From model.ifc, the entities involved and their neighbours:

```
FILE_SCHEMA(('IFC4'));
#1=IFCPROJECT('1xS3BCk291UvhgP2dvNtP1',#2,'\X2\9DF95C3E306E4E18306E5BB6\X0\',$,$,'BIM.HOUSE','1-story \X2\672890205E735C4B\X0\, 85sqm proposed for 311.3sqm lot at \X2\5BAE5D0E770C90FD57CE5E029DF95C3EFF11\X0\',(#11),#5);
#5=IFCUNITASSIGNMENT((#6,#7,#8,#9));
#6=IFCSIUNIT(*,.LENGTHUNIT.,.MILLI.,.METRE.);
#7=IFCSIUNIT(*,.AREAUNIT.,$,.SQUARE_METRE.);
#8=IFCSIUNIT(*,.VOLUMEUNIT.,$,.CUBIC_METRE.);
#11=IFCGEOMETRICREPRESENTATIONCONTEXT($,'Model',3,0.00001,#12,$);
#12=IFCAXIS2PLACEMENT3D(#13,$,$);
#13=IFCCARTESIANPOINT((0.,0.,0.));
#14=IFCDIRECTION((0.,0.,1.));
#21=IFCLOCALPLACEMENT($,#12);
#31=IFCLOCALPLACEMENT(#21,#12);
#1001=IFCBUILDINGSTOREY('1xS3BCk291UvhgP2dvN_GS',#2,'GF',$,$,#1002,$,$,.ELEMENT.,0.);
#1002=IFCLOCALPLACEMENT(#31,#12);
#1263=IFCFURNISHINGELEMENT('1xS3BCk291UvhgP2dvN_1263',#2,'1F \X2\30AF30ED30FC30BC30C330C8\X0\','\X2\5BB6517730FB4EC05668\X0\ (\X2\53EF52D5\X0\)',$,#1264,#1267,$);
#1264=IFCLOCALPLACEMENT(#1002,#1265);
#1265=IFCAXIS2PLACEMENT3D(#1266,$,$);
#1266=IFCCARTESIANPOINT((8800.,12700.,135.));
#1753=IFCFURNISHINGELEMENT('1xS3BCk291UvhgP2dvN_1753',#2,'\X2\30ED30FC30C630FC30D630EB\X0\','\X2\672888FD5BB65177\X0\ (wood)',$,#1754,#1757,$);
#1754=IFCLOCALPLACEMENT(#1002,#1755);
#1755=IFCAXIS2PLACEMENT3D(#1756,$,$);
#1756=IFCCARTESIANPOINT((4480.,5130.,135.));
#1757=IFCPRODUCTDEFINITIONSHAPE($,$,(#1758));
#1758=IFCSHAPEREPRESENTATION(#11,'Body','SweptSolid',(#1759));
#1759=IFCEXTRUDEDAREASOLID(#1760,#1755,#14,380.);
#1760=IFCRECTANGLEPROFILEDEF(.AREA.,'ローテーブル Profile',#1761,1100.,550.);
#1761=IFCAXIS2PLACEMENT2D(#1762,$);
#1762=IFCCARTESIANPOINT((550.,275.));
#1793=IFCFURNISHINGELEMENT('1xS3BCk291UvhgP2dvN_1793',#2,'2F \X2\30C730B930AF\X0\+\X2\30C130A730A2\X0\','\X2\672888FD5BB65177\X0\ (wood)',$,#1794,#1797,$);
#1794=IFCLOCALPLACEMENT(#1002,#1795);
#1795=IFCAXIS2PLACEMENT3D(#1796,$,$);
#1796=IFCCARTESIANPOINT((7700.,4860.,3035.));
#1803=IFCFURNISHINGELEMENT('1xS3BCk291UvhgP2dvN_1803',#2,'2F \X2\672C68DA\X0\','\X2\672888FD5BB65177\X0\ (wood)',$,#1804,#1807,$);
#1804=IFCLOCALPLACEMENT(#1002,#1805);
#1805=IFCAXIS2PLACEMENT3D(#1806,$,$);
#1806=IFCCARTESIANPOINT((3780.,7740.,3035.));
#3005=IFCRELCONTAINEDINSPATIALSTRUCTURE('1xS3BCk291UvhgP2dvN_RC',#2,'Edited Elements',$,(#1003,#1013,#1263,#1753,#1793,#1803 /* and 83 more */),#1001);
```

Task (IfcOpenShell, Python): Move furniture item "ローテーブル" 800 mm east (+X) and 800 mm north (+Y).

```python
import ifcopenshell
import ifcopenshell.api.geometry
import ifcopenshell.util.placement
import ifcopenshell.util.unit

model = ifcopenshell.open("model.ifc")
unit_scale = ifcopenshell.util.unit.calculate_unit_scale(model)

item = model.by_guid("1xS3BCk291UvhgP2dvN_1753")
matrix = ifcopenshell.util.placement.get_local_placement(item.ObjectPlacement)
matrix[0, 3] += 0.8 / unit_scale
matrix[1, 3] += 0.8 / unit_scale
ifcopenshell.api.geometry.edit_object_placement(model, product=item, matrix=matrix, is_si=False)

print(ifcopenshell.util.placement.get_local_placement(item.ObjectPlacement).round(3) + 0.0)

model.write("model_edited.ifc")
```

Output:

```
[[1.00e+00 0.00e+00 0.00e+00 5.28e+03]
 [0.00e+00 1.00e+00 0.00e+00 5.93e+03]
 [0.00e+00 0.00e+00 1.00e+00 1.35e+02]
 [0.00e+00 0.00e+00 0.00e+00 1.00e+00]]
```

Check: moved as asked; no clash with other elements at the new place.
